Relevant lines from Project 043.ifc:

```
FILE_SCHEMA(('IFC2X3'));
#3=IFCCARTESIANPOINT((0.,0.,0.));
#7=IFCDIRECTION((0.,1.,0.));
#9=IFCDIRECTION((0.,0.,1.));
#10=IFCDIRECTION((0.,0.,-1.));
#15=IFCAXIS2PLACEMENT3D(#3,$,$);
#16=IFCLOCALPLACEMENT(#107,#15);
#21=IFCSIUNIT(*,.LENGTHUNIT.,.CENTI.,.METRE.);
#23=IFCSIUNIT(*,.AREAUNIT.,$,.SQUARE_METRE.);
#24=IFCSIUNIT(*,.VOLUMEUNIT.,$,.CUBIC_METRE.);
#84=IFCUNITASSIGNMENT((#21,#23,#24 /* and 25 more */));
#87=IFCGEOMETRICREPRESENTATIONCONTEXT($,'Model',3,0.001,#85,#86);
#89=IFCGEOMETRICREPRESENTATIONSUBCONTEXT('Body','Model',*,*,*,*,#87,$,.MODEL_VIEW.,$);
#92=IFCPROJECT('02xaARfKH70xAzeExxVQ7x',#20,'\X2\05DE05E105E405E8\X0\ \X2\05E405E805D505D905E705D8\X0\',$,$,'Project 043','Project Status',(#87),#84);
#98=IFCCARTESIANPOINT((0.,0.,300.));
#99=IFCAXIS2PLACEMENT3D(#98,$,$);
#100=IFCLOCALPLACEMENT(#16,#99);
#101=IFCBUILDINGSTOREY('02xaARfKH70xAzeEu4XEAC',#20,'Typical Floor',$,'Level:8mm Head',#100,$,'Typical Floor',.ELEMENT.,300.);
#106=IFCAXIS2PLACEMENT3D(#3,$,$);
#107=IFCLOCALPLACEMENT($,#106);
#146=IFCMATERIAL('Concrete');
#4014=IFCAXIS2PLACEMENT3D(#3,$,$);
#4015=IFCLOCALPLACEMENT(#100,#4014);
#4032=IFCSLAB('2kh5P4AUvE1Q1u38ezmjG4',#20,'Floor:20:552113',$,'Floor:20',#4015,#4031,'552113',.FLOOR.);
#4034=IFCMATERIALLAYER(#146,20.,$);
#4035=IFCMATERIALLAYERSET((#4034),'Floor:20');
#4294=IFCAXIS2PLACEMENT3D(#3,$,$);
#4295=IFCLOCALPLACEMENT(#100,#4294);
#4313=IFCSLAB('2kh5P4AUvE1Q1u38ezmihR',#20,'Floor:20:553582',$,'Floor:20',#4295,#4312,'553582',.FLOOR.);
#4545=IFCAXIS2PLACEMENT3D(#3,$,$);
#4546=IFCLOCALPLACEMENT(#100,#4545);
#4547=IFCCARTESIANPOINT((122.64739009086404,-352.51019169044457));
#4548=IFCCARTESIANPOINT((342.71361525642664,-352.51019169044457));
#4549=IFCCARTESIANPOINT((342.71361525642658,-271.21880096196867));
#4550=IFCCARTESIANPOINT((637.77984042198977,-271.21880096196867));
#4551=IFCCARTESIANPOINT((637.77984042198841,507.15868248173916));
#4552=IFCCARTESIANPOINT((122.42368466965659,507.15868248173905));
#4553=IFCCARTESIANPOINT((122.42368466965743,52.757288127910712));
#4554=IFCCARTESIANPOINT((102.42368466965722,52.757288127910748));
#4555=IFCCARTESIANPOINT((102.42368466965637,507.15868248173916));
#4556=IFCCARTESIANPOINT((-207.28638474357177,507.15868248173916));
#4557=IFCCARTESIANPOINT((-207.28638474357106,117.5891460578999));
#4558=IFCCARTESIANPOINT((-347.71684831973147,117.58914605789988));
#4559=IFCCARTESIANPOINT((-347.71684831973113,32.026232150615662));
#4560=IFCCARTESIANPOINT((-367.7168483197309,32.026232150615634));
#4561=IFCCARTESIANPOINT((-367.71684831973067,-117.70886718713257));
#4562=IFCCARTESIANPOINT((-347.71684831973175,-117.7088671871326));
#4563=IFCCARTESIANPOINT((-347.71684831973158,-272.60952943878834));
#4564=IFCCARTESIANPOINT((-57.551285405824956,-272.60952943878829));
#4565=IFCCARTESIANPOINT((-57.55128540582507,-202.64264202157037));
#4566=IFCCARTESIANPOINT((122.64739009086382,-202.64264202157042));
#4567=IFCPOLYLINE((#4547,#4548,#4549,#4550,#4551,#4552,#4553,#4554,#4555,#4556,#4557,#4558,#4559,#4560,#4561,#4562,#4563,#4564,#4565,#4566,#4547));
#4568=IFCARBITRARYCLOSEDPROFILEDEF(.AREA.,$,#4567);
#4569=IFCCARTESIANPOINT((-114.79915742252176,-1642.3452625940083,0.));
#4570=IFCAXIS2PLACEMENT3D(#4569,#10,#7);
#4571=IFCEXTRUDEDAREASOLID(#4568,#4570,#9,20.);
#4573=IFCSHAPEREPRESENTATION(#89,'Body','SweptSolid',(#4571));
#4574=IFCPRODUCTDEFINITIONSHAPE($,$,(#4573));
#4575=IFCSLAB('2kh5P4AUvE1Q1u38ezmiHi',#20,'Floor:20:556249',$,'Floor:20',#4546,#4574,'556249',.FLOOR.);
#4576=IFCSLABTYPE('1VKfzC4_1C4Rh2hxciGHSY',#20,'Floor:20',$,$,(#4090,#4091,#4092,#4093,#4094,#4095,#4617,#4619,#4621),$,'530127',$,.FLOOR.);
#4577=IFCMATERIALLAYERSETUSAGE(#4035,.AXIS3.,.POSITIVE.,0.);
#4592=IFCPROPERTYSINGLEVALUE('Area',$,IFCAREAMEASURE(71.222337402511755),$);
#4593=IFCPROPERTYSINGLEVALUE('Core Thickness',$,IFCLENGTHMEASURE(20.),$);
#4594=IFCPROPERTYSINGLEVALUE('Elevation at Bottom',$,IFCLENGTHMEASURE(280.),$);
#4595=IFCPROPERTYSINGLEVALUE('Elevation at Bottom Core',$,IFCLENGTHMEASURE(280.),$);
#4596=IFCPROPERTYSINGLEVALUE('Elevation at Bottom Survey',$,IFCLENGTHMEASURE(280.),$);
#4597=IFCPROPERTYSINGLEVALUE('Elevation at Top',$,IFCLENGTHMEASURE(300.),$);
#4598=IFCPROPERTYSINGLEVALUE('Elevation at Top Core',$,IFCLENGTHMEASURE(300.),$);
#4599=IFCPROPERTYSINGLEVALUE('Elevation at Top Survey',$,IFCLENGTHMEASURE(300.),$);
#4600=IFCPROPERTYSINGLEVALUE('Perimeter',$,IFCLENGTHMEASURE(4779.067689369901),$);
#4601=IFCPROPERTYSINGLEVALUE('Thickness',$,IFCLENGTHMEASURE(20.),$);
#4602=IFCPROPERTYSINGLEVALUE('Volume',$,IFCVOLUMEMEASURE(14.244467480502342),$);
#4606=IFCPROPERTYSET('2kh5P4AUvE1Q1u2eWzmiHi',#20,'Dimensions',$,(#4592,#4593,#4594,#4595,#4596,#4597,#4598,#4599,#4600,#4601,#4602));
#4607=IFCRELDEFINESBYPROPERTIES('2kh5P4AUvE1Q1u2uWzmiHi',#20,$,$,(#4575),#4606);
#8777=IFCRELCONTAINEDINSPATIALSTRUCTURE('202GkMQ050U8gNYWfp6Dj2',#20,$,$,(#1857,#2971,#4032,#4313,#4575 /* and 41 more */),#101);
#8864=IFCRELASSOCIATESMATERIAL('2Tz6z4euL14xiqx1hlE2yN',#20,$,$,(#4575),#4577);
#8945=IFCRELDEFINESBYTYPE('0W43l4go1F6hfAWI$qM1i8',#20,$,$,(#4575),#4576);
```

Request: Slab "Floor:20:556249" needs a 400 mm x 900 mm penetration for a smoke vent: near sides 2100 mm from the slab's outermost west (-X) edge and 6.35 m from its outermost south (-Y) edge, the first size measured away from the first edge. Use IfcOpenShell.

```python
import numpy as np
import ifcopenshell
import ifcopenshell.api.feature
import ifcopenshell.api.geometry
import ifcopenshell.api.pset
import ifcopenshell.api.root
import ifcopenshell.geom
import ifcopenshell.util.element
import ifcopenshell.util.placement
import ifcopenshell.util.representation
import ifcopenshell.util.shape
import ifcopenshell.util.unit

model = ifcopenshell.open("Project 043.ifc")
unit_scale = ifcopenshell.util.unit.calculate_unit_scale(model)
area_scale = ifcopenshell.util.unit.calculate_unit_scale(model, "AREAUNIT")
volume_scale = ifcopenshell.util.unit.calculate_unit_scale(model, "VOLUMEUNIT")
settings = ifcopenshell.geom.settings()


def volume(element):
    """Net volume in cubic metres, openings subtracted."""
    shape = ifcopenshell.geom.create_shape(settings, element)
    return ifcopenshell.util.shape.get_volume(shape.geometry)


slab = model.by_id(4575)
before = volume(slab)

# Extent in the slab's own axes, in metres. The edges named are its -X and -Y sides.
slab_shape = ifcopenshell.geom.create_shape(settings, slab)
vertices = ifcopenshell.util.shape.get_vertices(slab_shape.geometry)
x_min, y_min, bottom = vertices.min(axis=0)
top = vertices[:, 2].max()

opening = ifcopenshell.api.root.create_entity(model, ifc_class="IfcOpeningElement", name="Smoke vent opening")
context = ifcopenshell.util.representation.get_context(model, "Model", "Body", "MODEL_VIEW")
width, depth = 0.4, 0.9
outline = [(0.0, 0.0), (width, 0.0), (width, depth), (0.0, depth), (0.0, 0.0)]
# Overshoot both faces by 50 mm so the cut is clean.
shape = ifcopenshell.api.geometry.add_slab_representation(
    model, context=context, depth=top - bottom + 0.1, polyline=outline
)
ifcopenshell.api.geometry.assign_representation(model, product=opening, representation=shape)

matrix = ifcopenshell.util.placement.get_local_placement(slab.ObjectPlacement)
matrix[:, 3] = matrix @ np.append(np.array([x_min + 2.1, y_min + 6.35, bottom - 0.05]) / unit_scale, 1.0)
ifcopenshell.api.geometry.edit_object_placement(model, product=opening, matrix=matrix, is_si=False)
ifcopenshell.api.feature.add_feature(model, feature=opening, element=slab)

after = volume(slab)

# Update the slab's stored quantities.
pset = model.by_id(ifcopenshell.util.element.get_pset(slab, "Dimensions", should_inherit=False)["id"])
ifcopenshell.api.pset.edit_pset(model, pset=pset, properties={
    "Area": model.create_entity("IfcAreaMeasure", after / (top - bottom) / area_scale),
    "Volume": model.create_entity("IfcVolumeMeasure", after / volume_scale),
})

print(f"slab volume {before:.3f} -> {after:.3f} m3")

model.write("Project 043_v2.ifc")
```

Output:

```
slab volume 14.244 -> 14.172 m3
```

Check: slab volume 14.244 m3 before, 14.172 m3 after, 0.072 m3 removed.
